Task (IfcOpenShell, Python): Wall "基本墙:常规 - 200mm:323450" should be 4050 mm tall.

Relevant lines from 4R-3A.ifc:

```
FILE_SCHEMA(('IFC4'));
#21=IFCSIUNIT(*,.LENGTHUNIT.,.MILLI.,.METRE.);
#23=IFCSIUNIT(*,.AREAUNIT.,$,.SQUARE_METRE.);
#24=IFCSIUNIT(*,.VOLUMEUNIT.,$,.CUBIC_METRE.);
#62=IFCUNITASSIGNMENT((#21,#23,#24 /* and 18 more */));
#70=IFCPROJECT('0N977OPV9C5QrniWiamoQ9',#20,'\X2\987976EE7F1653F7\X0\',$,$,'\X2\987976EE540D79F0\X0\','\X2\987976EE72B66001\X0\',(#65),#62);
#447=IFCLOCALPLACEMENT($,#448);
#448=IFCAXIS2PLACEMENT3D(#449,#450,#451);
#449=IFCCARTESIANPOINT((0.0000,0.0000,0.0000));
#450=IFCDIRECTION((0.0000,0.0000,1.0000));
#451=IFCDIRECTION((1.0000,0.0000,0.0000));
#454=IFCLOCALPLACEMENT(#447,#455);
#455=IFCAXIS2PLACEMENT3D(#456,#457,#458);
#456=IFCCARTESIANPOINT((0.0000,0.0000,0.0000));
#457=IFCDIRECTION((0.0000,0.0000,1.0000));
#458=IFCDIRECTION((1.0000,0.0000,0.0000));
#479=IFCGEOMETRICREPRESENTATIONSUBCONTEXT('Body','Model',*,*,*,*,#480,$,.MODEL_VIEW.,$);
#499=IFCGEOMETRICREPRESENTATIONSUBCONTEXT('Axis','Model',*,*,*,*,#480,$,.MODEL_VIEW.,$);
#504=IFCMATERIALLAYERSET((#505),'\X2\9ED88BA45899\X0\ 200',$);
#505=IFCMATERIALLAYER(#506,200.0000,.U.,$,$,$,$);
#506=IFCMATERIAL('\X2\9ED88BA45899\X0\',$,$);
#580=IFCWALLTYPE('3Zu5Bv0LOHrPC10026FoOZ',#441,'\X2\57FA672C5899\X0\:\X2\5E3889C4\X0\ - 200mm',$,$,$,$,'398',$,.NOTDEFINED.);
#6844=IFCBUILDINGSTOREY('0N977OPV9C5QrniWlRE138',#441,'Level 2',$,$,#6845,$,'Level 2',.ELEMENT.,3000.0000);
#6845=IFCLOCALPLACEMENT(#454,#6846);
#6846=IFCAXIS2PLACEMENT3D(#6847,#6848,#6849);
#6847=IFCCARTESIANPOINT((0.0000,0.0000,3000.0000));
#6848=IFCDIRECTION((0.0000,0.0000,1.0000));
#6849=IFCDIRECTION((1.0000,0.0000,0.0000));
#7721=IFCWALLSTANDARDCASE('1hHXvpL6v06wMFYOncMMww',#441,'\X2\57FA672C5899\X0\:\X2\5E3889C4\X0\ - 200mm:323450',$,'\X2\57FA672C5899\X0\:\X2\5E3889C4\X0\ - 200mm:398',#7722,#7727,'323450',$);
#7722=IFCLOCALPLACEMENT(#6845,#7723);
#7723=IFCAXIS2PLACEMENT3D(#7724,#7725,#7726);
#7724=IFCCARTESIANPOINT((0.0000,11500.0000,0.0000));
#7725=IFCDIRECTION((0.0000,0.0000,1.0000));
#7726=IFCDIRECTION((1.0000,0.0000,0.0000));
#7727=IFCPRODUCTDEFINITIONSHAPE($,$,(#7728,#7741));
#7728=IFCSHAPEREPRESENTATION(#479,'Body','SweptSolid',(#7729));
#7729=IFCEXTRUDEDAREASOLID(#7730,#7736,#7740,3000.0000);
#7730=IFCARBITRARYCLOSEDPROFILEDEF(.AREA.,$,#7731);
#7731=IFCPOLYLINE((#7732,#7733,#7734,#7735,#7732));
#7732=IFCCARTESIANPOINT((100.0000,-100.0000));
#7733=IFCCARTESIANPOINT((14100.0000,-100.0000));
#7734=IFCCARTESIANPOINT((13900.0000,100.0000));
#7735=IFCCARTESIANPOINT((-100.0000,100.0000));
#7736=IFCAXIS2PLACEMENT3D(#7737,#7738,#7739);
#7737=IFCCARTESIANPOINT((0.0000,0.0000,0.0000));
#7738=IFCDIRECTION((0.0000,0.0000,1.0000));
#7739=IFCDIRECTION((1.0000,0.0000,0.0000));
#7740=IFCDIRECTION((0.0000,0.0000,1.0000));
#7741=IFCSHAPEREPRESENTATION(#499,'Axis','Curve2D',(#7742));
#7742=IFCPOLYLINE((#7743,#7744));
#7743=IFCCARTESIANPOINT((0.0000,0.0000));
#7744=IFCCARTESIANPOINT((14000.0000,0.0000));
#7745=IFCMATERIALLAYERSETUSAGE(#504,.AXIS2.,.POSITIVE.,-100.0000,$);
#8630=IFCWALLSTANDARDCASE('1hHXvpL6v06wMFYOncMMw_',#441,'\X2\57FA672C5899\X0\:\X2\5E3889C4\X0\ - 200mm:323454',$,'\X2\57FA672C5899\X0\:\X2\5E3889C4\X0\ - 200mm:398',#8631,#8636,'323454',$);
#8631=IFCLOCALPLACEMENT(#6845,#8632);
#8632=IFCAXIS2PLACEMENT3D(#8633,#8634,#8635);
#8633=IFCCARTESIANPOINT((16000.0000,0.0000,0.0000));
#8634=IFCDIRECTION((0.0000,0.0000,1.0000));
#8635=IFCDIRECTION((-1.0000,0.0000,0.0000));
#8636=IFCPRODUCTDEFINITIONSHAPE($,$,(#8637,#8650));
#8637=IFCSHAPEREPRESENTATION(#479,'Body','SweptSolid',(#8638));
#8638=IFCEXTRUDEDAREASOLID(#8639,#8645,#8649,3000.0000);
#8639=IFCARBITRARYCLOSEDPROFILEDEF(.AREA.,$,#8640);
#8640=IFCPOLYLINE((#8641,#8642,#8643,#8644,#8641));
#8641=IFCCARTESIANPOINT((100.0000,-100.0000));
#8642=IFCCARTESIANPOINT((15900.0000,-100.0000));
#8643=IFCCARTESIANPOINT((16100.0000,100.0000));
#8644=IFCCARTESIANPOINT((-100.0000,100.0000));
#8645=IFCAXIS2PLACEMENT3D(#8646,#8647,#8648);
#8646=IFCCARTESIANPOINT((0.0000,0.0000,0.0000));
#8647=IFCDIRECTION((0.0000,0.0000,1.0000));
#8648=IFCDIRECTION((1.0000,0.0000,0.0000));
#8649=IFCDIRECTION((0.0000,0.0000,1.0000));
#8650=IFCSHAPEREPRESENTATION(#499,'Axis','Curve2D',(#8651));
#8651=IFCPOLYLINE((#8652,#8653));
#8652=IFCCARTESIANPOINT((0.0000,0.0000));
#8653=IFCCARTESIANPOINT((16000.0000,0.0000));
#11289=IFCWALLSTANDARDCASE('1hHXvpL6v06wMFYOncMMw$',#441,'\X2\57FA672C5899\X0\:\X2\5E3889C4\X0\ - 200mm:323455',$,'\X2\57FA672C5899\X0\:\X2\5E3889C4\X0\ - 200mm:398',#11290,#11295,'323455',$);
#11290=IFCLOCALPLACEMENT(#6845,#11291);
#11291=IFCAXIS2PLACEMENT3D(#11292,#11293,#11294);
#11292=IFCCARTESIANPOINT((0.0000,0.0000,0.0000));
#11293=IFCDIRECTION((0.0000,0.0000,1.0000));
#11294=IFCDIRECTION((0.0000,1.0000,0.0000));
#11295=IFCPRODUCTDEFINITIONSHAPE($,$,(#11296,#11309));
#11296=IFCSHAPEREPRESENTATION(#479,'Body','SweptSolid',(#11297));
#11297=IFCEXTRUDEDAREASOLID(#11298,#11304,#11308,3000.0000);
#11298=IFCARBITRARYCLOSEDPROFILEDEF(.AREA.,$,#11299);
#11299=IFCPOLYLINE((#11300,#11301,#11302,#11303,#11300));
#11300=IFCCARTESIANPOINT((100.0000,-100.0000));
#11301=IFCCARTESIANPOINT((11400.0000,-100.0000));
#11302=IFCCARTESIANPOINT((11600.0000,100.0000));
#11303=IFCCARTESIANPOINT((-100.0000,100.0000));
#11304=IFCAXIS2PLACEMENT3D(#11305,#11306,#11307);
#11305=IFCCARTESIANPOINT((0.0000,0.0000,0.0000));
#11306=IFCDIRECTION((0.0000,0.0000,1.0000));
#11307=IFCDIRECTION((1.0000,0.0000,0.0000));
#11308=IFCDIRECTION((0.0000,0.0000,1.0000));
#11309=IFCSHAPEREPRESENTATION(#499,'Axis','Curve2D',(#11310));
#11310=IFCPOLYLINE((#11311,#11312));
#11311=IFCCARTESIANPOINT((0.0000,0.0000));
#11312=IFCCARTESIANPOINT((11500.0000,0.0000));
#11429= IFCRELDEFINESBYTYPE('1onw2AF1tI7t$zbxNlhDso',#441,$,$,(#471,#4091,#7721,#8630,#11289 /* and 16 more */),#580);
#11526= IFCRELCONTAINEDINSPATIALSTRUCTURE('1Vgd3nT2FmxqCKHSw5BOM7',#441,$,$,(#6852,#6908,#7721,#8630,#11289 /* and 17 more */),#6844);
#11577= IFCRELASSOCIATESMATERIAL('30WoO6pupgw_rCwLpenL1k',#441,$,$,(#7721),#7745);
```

```python
import ifcopenshell
import ifcopenshell.geom
import ifcopenshell.util.representation
import ifcopenshell.util.shape
import ifcopenshell.util.unit

model = ifcopenshell.open("4R-3A.ifc")
unit_scale = ifcopenshell.util.unit.calculate_unit_scale(model)
settings = ifcopenshell.geom.settings()


def volume(element):
    """Net volume in cubic metres, openings subtracted."""
    shape = ifcopenshell.geom.create_shape(settings, element)
    return ifcopenshell.util.shape.get_volume(shape.geometry)


wall = model.by_guid("1hHXvpL6v06wMFYOncMMww")
before = volume(wall)

body = ifcopenshell.util.representation.get_representation(wall, "Model", "Body")
solid = body.Items[0]
old_height = solid.Depth
solid.Depth = 4.05 / unit_scale
after = volume(wall)

print(f"height {old_height:g} -> {solid.Depth:g}, volume {before:.3f} -> {after:.3f} m3")

model.write("4R-3A_v2.ifc")
```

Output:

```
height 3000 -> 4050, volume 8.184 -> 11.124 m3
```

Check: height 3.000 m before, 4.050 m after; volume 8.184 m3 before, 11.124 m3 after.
